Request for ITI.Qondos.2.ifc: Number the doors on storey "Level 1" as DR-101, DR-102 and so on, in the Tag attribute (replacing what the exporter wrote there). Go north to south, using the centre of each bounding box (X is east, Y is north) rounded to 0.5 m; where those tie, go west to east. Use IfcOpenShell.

First a look at what the model holds.

```python
import ifcopenshell
import ifcopenshell.util.element
import ifcopenshell.util.placement

model = ifcopenshell.open("ITI.Qondos.2.ifc")
print(model.schema)
storey = next(s for s in model.by_type("IfcBuildingStorey") if s.Name == "Level 1")
doors = [e for e in ifcopenshell.util.element.get_decomposition(storey) if e.is_a("IfcDoor")]
for e in sorted(doors, key=lambda e: e.id()):
    origin = ifcopenshell.util.placement.get_local_placement(e.ObjectPlacement)[:3, 3]
    print(e.id(), e.Tag, e.Name, origin.round(2) + 0.0, sep=" | ")
```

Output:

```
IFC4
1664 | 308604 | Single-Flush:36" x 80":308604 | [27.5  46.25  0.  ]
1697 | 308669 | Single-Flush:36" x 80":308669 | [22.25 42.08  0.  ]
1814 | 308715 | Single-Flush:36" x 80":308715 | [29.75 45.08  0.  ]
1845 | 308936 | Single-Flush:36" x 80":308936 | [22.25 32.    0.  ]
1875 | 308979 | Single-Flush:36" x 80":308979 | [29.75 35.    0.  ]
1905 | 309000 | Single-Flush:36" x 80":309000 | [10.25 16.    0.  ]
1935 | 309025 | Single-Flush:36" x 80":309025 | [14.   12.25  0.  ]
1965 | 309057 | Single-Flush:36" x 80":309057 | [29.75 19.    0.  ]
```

```python
import ifcopenshell
import ifcopenshell.geom
import ifcopenshell.util.element
import ifcopenshell.util.shape

model = ifcopenshell.open("ITI.Qondos.2.ifc")
settings = ifcopenshell.geom.settings()
settings.set("use-world-coords", True)


def centre(element):
    shape = ifcopenshell.geom.create_shape(settings, element)
    return ifcopenshell.util.shape.get_bbox_centroid(shape.geometry)


storey = next(s for s in model.by_type("IfcBuildingStorey") if s.Name == "Level 1")
doors = [e for e in ifcopenshell.util.element.get_decomposition(storey) if e.is_a("IfcDoor")]

# Insertion points can sit at a corner or the storey origin, so sort by the geometry (in metres).
centres = {e: centre(e) for e in doors}
doors.sort(key=lambda e: (-round(centres[e][1] / 0.5), centres[e][0]))

for i, e in enumerate(doors, start=1):
    number = f"DR-1{i:02d}"
    e.Tag = number
    print(e.id(), number)

model.write("ITI.Qondos.2_updated.ifc")
```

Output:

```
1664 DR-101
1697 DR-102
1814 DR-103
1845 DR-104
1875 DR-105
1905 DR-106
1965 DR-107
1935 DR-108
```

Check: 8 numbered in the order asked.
